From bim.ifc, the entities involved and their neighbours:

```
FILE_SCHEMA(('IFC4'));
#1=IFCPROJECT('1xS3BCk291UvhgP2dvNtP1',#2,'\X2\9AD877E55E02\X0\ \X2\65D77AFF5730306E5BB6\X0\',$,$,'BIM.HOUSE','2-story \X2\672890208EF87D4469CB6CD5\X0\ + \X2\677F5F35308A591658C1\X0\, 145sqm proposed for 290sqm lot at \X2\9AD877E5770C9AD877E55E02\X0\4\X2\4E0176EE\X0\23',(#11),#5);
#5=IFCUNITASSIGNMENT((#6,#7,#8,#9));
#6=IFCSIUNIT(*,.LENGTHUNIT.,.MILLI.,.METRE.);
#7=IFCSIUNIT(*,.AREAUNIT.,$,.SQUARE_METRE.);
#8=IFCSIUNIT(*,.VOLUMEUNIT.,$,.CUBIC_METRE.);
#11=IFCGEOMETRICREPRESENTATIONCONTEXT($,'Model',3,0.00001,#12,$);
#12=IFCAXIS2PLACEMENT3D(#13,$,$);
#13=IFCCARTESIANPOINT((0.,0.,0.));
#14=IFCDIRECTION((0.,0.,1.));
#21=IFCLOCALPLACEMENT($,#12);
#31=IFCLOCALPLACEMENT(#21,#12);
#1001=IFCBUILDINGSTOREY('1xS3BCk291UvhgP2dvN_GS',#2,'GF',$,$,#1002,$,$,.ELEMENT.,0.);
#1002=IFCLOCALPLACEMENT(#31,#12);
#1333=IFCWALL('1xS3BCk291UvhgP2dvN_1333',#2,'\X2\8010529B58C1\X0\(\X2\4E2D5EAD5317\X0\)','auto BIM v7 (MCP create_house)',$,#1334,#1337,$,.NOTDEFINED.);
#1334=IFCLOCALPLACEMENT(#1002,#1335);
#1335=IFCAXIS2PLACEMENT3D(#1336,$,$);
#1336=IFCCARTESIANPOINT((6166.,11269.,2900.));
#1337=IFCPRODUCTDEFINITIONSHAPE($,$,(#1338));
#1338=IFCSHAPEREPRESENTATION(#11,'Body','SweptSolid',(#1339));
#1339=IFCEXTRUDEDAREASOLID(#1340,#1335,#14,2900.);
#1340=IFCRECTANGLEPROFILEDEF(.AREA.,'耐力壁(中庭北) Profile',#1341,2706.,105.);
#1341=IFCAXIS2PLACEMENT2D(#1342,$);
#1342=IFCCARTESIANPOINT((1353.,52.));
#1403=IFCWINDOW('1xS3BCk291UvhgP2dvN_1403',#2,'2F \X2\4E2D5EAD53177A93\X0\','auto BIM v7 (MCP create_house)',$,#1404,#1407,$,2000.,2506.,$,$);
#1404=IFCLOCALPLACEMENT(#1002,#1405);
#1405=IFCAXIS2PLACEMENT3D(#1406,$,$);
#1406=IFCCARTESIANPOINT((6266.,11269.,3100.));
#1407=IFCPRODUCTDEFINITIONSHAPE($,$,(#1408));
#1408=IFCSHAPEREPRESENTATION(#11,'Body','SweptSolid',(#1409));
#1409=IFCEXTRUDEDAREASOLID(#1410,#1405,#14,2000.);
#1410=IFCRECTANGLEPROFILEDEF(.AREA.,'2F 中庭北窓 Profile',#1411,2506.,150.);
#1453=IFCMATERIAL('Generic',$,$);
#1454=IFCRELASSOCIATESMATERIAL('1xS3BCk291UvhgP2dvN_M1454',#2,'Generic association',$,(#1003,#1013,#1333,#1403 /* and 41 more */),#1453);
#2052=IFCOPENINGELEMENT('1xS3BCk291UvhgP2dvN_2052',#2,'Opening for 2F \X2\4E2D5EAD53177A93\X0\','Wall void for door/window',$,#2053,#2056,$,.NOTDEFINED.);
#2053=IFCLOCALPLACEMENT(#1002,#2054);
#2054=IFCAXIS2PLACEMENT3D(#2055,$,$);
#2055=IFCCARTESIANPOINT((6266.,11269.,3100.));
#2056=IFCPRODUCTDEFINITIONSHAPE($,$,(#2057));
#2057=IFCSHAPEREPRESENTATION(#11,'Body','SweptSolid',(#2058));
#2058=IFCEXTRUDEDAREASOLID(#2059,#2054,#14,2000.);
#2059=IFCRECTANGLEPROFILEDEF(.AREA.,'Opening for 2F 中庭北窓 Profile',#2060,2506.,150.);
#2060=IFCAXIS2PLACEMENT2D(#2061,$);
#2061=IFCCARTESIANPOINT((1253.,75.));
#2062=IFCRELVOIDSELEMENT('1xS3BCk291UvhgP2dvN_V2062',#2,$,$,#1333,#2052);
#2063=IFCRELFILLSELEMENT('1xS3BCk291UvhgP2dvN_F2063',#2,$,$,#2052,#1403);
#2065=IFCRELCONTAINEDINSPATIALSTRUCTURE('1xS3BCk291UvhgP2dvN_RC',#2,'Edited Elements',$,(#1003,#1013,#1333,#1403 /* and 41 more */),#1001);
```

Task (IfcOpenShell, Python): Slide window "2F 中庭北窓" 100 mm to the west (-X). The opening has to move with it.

```python
import ifcopenshell
import ifcopenshell.api.geometry
import ifcopenshell.util.placement
import ifcopenshell.util.unit

model = ifcopenshell.open("bim.ifc")
unit_scale = ifcopenshell.util.unit.calculate_unit_scale(model)

window = model.by_guid("1xS3BCk291UvhgP2dvN_1403")
opening = window.FillsVoids[0].RelatingOpeningElement
wall = opening.VoidsElements[0].RelatingBuildingElement

wall_matrix = ifcopenshell.util.placement.get_local_placement(wall.ObjectPlacement)
shift = wall_matrix[:3, 0] * -0.1 / unit_scale
before = ifcopenshell.util.placement.get_local_placement(window.ObjectPlacement)[:3, 3].copy()

# The window is not placed relative to its opening, so move both.
for product in (opening, window):
    matrix = ifcopenshell.util.placement.get_local_placement(product.ObjectPlacement)
    matrix[:3, 3] += shift
    ifcopenshell.api.geometry.edit_object_placement(model, product=product, matrix=matrix, is_si=False)

after = ifcopenshell.util.placement.get_local_placement(window.ObjectPlacement)[:3, 3]
print("window moved by", (after - before).round(3) + 0.0)

model.write("bim_v2.ifc")
```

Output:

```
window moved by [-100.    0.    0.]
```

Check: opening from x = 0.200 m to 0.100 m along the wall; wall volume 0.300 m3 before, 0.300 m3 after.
